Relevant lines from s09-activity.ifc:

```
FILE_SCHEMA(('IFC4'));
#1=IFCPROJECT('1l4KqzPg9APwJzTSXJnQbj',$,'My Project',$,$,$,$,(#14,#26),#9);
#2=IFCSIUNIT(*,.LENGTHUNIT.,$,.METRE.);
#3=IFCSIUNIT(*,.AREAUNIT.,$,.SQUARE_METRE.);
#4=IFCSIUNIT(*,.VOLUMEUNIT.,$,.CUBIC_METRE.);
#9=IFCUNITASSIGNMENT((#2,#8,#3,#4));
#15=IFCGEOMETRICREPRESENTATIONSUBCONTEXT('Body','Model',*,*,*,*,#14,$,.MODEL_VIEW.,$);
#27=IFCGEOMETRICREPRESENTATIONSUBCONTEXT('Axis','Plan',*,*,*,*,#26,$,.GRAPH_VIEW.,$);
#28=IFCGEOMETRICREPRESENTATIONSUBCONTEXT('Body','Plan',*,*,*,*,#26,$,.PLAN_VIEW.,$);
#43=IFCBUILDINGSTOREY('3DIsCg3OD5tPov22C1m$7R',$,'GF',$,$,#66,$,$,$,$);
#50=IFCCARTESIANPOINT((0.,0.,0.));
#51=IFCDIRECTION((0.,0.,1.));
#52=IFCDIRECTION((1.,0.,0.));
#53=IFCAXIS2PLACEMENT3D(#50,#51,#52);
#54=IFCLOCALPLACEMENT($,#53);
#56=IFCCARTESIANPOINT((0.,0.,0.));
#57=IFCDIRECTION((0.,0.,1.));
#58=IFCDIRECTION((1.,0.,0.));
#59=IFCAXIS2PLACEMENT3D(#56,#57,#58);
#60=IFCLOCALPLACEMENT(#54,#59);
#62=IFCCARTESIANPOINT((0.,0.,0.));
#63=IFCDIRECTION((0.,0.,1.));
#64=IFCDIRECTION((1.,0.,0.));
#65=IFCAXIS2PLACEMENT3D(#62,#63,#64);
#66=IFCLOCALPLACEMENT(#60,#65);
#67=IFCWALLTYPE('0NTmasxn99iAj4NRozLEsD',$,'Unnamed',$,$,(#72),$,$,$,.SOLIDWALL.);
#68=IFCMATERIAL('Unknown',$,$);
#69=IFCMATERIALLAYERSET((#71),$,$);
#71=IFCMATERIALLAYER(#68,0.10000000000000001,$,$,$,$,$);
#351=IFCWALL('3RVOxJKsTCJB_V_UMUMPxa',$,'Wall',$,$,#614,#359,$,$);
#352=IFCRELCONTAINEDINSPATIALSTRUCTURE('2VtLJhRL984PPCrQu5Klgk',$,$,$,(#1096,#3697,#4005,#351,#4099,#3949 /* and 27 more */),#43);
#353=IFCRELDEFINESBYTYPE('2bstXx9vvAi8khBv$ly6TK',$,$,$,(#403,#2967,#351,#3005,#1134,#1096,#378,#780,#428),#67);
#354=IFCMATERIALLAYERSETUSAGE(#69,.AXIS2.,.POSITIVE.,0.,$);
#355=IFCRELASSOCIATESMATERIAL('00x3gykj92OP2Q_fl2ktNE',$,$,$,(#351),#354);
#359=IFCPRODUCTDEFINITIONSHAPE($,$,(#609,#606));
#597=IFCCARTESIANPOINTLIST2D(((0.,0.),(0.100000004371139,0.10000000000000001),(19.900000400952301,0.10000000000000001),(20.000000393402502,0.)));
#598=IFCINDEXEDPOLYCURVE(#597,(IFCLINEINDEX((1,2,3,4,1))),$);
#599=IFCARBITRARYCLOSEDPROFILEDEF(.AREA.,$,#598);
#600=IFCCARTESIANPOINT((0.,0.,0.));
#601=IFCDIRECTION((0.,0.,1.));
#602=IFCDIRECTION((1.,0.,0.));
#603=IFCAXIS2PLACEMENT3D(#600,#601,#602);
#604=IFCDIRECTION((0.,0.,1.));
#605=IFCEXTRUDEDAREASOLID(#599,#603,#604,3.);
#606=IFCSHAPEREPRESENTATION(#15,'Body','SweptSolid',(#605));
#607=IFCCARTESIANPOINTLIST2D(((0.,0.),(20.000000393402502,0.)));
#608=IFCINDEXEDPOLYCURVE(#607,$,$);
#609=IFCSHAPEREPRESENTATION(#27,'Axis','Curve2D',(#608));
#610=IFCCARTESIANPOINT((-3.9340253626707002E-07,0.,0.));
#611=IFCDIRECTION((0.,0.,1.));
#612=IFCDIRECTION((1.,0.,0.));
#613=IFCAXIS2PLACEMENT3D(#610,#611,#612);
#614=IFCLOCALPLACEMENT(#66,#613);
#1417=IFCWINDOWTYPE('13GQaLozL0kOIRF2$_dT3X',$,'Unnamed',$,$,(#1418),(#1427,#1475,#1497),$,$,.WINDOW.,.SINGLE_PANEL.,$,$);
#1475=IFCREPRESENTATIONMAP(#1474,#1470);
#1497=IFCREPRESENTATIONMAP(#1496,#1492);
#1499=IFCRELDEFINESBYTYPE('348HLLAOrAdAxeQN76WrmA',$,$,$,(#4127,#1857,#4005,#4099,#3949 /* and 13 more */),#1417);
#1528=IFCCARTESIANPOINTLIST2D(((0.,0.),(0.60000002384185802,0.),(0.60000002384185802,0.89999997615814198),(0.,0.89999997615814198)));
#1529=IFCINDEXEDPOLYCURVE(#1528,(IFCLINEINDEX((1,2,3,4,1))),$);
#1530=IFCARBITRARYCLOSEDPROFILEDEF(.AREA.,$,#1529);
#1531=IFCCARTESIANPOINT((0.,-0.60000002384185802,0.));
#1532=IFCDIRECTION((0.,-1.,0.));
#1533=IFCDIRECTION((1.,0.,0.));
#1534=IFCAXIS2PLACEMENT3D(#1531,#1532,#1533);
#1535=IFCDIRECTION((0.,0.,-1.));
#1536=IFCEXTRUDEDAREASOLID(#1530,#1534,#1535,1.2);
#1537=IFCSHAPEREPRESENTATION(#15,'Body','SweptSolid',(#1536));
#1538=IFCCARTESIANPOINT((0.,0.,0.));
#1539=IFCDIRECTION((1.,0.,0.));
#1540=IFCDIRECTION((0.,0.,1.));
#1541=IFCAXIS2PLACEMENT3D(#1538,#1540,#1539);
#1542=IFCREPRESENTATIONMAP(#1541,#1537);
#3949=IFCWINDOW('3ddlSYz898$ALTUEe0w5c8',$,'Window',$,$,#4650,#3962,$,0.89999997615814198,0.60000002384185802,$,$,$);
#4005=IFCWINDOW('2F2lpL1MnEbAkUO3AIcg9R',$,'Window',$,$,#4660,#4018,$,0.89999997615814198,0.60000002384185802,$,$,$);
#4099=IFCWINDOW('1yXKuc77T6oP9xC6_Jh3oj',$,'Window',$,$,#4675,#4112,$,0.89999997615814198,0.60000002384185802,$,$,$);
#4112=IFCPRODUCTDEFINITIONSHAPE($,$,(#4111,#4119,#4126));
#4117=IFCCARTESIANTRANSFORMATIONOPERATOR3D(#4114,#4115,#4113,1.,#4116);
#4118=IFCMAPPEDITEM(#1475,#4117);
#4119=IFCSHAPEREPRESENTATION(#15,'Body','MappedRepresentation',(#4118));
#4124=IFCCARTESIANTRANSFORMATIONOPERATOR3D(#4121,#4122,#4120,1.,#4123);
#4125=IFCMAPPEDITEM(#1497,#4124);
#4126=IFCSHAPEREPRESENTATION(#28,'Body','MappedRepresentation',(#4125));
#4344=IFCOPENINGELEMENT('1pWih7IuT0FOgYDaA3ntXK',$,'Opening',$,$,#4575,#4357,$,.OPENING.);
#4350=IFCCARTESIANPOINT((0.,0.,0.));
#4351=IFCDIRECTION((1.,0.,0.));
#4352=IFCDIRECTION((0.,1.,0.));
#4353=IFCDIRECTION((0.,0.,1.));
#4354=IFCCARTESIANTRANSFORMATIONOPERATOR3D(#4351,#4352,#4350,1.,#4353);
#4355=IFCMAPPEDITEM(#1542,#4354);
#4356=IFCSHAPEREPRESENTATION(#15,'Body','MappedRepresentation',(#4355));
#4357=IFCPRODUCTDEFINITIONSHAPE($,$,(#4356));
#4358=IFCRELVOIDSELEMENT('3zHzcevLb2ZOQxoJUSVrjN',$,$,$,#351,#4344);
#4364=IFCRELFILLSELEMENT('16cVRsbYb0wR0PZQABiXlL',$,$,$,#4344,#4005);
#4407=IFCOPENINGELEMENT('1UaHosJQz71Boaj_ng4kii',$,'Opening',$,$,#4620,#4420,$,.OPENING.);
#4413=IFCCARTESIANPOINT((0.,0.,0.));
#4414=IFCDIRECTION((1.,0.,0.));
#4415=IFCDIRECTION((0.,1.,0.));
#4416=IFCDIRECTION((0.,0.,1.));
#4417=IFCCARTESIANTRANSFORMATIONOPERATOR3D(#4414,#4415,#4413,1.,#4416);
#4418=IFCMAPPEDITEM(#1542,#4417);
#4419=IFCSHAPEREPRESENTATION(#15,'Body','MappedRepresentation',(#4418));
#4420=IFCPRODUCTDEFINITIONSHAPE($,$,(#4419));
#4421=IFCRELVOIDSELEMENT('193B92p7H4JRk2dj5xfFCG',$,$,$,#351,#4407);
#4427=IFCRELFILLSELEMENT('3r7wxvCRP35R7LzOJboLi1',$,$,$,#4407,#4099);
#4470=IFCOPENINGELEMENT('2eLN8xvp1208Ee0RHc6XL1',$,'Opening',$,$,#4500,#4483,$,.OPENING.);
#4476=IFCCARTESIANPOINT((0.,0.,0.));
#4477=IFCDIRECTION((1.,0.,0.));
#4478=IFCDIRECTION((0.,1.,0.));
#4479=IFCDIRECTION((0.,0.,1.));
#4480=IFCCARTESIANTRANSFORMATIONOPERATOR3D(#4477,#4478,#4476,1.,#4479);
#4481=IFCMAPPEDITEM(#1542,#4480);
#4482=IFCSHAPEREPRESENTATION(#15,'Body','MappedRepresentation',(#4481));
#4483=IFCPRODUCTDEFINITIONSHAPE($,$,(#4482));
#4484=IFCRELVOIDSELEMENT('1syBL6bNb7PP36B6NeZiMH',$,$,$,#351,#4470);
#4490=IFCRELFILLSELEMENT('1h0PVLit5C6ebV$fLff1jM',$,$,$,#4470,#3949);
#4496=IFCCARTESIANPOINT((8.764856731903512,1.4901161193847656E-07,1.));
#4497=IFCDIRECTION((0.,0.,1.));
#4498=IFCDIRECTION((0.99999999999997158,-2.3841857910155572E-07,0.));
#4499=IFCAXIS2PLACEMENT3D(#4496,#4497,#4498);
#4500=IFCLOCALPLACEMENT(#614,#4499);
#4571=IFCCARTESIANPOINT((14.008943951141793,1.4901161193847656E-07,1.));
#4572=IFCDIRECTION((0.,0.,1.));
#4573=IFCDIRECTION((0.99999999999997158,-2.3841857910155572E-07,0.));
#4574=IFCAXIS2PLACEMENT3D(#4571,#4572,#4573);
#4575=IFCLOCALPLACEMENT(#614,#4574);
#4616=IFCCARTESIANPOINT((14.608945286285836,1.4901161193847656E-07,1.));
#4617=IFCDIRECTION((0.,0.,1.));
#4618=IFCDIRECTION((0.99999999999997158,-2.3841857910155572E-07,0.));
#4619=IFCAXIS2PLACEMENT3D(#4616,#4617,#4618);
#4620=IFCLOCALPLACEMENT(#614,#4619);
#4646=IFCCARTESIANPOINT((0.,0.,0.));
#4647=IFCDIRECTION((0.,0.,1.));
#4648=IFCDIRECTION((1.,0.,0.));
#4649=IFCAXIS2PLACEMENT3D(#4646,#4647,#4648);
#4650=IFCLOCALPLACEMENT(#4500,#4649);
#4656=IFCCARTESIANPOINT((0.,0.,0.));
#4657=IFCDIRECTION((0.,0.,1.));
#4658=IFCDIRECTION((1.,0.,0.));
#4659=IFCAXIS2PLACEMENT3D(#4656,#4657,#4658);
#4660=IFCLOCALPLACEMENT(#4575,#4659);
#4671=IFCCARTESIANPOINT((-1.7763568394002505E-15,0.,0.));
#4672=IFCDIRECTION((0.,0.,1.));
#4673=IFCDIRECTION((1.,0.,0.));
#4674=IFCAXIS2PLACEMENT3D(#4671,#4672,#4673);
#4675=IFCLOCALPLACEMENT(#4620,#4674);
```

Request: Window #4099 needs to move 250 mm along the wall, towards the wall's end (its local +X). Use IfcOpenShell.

```python
import ifcopenshell
import ifcopenshell.api.geometry
import ifcopenshell.util.placement

model = ifcopenshell.open("s09-activity.ifc")

window = model.by_guid("1yXKuc77T6oP9xC6_Jh3oj")
opening = window.FillsVoids[0].RelatingOpeningElement
wall = opening.VoidsElements[0].RelatingBuildingElement

wall_matrix = ifcopenshell.util.placement.get_local_placement(wall.ObjectPlacement)
shift = wall_matrix[:3, 0] * 0.25
before = ifcopenshell.util.placement.get_local_placement(window.ObjectPlacement)[:3, 3].copy()

# The window is placed relative to its opening, so it follows when the opening moves.
matrix = ifcopenshell.util.placement.get_local_placement(opening.ObjectPlacement)
matrix[:3, 3] += shift
ifcopenshell.api.geometry.edit_object_placement(
    model, product=opening, matrix=matrix, is_si=False, should_transform_children=True
)

after = ifcopenshell.util.placement.get_local_placement(window.ObjectPlacement)[:3, 3]
print("window moved by", (after - before).round(3) + 0.0)

model.write("s09-activity_edited.ifc")
```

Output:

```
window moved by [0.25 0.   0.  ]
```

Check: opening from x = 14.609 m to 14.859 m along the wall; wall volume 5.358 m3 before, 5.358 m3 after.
